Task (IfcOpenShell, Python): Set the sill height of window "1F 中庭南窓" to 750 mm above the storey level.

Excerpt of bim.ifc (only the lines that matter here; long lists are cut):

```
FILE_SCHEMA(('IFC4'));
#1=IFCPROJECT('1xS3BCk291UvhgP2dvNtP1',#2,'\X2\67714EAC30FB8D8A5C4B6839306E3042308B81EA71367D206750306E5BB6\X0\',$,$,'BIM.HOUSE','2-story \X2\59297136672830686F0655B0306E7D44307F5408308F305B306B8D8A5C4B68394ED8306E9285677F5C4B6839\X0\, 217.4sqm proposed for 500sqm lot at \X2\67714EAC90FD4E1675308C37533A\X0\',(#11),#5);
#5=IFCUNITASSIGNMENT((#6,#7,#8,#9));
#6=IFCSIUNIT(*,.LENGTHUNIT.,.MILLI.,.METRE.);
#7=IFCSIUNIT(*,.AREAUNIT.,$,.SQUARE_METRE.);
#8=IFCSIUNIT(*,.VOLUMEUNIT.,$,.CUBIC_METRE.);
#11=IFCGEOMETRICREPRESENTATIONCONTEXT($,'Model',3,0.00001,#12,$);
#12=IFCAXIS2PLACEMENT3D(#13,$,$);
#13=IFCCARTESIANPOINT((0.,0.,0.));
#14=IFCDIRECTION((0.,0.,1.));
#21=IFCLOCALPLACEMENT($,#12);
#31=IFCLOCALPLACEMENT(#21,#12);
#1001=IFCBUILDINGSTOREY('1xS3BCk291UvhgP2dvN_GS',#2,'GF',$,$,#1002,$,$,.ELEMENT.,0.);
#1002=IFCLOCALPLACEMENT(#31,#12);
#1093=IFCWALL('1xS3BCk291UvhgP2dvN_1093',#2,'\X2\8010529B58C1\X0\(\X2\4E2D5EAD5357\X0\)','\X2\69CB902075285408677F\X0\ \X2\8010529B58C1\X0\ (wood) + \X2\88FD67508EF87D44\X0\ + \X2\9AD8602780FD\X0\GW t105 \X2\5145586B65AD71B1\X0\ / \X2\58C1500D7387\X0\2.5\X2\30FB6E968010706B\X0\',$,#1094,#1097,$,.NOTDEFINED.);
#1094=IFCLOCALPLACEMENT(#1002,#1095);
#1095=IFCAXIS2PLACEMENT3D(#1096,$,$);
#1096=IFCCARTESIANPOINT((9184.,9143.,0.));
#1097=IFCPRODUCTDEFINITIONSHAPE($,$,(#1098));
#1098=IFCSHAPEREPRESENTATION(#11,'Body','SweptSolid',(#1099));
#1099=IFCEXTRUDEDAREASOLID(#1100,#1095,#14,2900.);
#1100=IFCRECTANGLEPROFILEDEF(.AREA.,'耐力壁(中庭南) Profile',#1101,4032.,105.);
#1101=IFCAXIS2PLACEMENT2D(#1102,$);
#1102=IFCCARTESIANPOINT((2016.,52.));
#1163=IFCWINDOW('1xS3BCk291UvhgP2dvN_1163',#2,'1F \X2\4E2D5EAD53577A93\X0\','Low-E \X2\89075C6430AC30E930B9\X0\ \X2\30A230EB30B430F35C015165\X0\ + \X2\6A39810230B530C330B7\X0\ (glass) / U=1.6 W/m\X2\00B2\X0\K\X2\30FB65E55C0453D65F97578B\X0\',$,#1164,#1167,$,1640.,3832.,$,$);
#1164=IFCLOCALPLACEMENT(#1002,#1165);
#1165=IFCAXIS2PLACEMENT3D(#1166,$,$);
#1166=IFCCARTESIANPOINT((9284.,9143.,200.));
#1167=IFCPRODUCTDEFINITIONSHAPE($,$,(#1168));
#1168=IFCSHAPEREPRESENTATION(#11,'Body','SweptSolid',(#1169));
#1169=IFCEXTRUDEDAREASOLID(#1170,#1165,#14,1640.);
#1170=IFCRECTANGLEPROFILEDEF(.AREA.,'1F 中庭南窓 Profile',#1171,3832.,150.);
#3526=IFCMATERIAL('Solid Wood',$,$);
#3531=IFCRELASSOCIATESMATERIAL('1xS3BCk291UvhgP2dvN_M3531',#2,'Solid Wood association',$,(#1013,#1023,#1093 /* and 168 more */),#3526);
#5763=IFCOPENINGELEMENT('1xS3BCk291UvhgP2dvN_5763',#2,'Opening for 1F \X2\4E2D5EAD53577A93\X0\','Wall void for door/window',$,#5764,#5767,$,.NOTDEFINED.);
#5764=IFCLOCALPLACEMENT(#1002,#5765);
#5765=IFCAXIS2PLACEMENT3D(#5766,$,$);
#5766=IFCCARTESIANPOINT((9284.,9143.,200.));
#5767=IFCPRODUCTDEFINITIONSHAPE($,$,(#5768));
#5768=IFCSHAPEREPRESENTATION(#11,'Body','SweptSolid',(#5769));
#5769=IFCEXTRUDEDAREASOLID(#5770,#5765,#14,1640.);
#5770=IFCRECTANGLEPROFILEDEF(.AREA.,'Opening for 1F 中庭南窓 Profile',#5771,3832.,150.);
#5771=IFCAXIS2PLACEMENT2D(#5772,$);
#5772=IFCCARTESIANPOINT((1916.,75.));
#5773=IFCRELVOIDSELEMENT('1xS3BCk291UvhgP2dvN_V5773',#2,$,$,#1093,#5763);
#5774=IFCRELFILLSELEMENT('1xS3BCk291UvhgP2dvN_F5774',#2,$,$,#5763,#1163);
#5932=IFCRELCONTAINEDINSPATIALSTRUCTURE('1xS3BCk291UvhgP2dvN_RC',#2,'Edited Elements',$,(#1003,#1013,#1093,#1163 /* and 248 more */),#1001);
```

```python
import numpy as np
import ifcopenshell
import ifcopenshell.api.geometry
import ifcopenshell.geom
import ifcopenshell.util.element
import ifcopenshell.util.placement
import ifcopenshell.util.shape
import ifcopenshell.util.unit

model = ifcopenshell.open("bim.ifc")
unit_scale = ifcopenshell.util.unit.calculate_unit_scale(model)

window = model.by_guid("1xS3BCk291UvhgP2dvN_1163")
opening = window.FillsVoids[0].RelatingOpeningElement
storey = ifcopenshell.util.element.get_container(window, ifc_class="IfcBuildingStorey")
level = ifcopenshell.util.placement.get_local_placement(storey.ObjectPlacement)[2, 3]

# The opening's origin need not be at the sill, so measure its lowest point.
shape = ifcopenshell.geom.create_shape(ifcopenshell.geom.settings(), opening)
bottom = ifcopenshell.util.shape.get_shape_bottom_elevation(shape, shape.geometry) / unit_scale
dz = level + 0.75 / unit_scale - bottom

shift = np.array([0.0, 0.0, dz])
# The window is not placed relative to its opening, so move both.
for product in (opening, window):
    matrix = ifcopenshell.util.placement.get_local_placement(product.ObjectPlacement)
    matrix[:3, 3] += shift
    ifcopenshell.api.geometry.edit_object_placement(model, product=product, matrix=matrix, is_si=False)

print(f"moved by {dz * unit_scale:+.3f} m")

model.write("bim_edited.ifc")
```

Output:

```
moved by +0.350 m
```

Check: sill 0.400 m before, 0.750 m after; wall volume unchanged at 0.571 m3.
